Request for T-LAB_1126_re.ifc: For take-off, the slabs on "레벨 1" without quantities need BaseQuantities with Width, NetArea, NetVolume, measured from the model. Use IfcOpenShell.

First a look at what the model holds.

```python
import ifcopenshell
import ifcopenshell.util.element
import ifcopenshell.util.unit

model = ifcopenshell.open("T-LAB_1126_re.ifc")
print(model.schema)
for unit_type in ("LENGTHUNIT", "AREAUNIT", "VOLUMEUNIT"):
    print(unit_type, ifcopenshell.util.unit.calculate_unit_scale(model, unit_type))
storey = next(s for s in model.by_type("IfcBuildingStorey") if s.Name == "레벨 1")
slabs = [e for e in ifcopenshell.util.element.get_decomposition(storey) if e.is_a("IfcSlab")]
for e in sorted(slabs, key=lambda e: e.id()):
    print(e.id(), e.is_a(), e.Name, list(ifcopenshell.util.element.get_psets(e, qtos_only=True)), sep=" | ")
```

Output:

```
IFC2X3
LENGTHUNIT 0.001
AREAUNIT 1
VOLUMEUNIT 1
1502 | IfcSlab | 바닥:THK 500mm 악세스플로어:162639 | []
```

```python
import ifcopenshell
import ifcopenshell.api.pset
import ifcopenshell.geom
import ifcopenshell.util.element
import ifcopenshell.util.shape
import ifcopenshell.util.unit

model = ifcopenshell.open("T-LAB_1126_re.ifc")
unit_scale = ifcopenshell.util.unit.calculate_unit_scale(model)
area_scale = ifcopenshell.util.unit.calculate_unit_scale(model, "AREAUNIT")
volume_scale = ifcopenshell.util.unit.calculate_unit_scale(model, "VOLUMEUNIT")
settings = ifcopenshell.geom.settings()

storey = next(s for s in model.by_type("IfcBuildingStorey") if s.Name == "레벨 1")
slabs = [e for e in ifcopenshell.util.element.get_decomposition(storey) if e.is_a("IfcSlab")]

for e in sorted(slabs, key=lambda e: e.id()):
    if ifcopenshell.util.element.get_psets(e, qtos_only=True, should_inherit=False):
        continue
    # Geometry comes back in metres, in the element's own axes.
    shape = ifcopenshell.geom.create_shape(settings, e)
    values = {
        "Width": ifcopenshell.util.shape.get_z(shape.geometry) / unit_scale,
        "NetArea": ifcopenshell.util.shape.get_footprint_area(shape.geometry) / area_scale,
        "NetVolume": ifcopenshell.util.shape.get_volume(shape.geometry) / volume_scale,
    }
    qto = ifcopenshell.api.pset.add_qto(model, product=e, name="BaseQuantities")
    ifcopenshell.api.pset.edit_qto(model, qto=qto, properties=values)
    print(e.id(), {k: round(v, 3) for k, v in values.items()})

model.write("T-LAB_1126_re-out.ifc")
```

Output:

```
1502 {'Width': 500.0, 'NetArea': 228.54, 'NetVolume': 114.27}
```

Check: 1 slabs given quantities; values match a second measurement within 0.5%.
